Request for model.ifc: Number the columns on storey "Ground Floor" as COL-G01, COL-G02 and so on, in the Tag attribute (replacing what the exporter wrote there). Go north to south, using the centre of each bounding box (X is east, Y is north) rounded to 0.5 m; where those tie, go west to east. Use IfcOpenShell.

First a look at what the model holds.

```python
import ifcopenshell
import ifcopenshell.util.element
import ifcopenshell.util.placement

model = ifcopenshell.open("model.ifc")
print(model.schema)
storey = next(s for s in model.by_type("IfcBuildingStorey") if s.Name == "Ground Floor")
columns = [e for e in ifcopenshell.util.element.get_decomposition(storey) if e.is_a("IfcColumn")]
for e in sorted(columns, key=lambda e: e.id()):
    origin = ifcopenshell.util.placement.get_local_placement(e.ObjectPlacement)[:3, 3]
    print(e.id(), e.Tag, e.Name, origin.round(2) + 0.0, sep=" | ")
```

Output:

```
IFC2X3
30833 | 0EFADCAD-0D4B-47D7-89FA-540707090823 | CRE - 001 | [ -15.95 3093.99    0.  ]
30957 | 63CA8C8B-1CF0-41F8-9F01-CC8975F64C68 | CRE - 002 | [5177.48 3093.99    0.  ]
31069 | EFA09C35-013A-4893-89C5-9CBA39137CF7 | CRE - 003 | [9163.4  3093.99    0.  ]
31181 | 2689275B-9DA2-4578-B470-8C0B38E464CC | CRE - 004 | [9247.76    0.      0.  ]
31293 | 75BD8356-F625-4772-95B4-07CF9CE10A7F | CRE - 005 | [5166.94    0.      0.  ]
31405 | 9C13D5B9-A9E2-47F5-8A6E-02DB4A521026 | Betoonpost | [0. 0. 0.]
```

```python
import ifcopenshell
import ifcopenshell.geom
import ifcopenshell.util.element
import ifcopenshell.util.shape

model = ifcopenshell.open("model.ifc")
settings = ifcopenshell.geom.settings()
settings.set("use-world-coords", True)


def centre(element):
    shape = ifcopenshell.geom.create_shape(settings, element)
    return ifcopenshell.util.shape.get_bbox_centroid(shape.geometry)


storey = next(s for s in model.by_type("IfcBuildingStorey") if s.Name == "Ground Floor")
columns = [e for e in ifcopenshell.util.element.get_decomposition(storey) if e.is_a("IfcColumn")]

# Insertion points can sit at a corner or the storey origin, so sort by the geometry (in metres).
centres = {e: centre(e) for e in columns}
columns.sort(key=lambda e: (-round(centres[e][1] / 0.5), centres[e][0]))

for i, e in enumerate(columns, start=1):
    number = f"COL-G{i:02d}"
    e.Tag = number
    print(e.id(), number)

model.write("model_v2.ifc")
```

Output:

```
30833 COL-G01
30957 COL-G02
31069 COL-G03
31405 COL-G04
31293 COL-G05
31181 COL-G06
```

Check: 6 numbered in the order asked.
